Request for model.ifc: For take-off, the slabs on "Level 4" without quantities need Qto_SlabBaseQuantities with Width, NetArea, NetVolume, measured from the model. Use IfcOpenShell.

First a look at what the model holds.

```python
import ifcopenshell
import ifcopenshell.util.element
import ifcopenshell.util.unit

model = ifcopenshell.open("model.ifc")
print(model.schema)
for unit_type in ("LENGTHUNIT", "AREAUNIT", "VOLUMEUNIT"):
    print(unit_type, ifcopenshell.util.unit.calculate_unit_scale(model, unit_type))
storey = next(s for s in model.by_type("IfcBuildingStorey") if s.Name == "Level 4")
slabs = [e for e in ifcopenshell.util.element.get_decomposition(storey) if e.is_a("IfcSlab")]
for e in sorted(slabs, key=lambda e: e.id()):
    print(e.id(), e.is_a(), e.Name, list(ifcopenshell.util.element.get_psets(e, qtos_only=True)), sep=" | ")
```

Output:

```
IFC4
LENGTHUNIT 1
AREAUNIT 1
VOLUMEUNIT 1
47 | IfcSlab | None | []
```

```python
import ifcopenshell
import ifcopenshell.api.pset
import ifcopenshell.geom
import ifcopenshell.util.element
import ifcopenshell.util.shape
import ifcopenshell.util.unit

model = ifcopenshell.open("model.ifc")
unit_scale = ifcopenshell.util.unit.calculate_unit_scale(model)
area_scale = ifcopenshell.util.unit.calculate_unit_scale(model, "AREAUNIT")
volume_scale = ifcopenshell.util.unit.calculate_unit_scale(model, "VOLUMEUNIT")
settings = ifcopenshell.geom.settings()

storey = next(s for s in model.by_type("IfcBuildingStorey") if s.Name == "Level 4")
slabs = [e for e in ifcopenshell.util.element.get_decomposition(storey) if e.is_a("IfcSlab")]

for e in sorted(slabs, key=lambda e: e.id()):
    if ifcopenshell.util.element.get_psets(e, qtos_only=True, should_inherit=False):
        continue
    # Geometry comes back in metres, in the element's own axes.
    shape = ifcopenshell.geom.create_shape(settings, e)
    values = {
        "Width": ifcopenshell.util.shape.get_z(shape.geometry) / unit_scale,
        "NetArea": ifcopenshell.util.shape.get_footprint_area(shape.geometry) / area_scale,
        "NetVolume": ifcopenshell.util.shape.get_volume(shape.geometry) / volume_scale,
    }
    qto = ifcopenshell.api.pset.add_qto(model, product=e, name="Qto_SlabBaseQuantities")
    ifcopenshell.api.pset.edit_qto(model, qto=qto, properties=values)
    print(e.id(), {k: round(v, 3) for k, v in values.items()})

model.write("model_updated.ifc")
```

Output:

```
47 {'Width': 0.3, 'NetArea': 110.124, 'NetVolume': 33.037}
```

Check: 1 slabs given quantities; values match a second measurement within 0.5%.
